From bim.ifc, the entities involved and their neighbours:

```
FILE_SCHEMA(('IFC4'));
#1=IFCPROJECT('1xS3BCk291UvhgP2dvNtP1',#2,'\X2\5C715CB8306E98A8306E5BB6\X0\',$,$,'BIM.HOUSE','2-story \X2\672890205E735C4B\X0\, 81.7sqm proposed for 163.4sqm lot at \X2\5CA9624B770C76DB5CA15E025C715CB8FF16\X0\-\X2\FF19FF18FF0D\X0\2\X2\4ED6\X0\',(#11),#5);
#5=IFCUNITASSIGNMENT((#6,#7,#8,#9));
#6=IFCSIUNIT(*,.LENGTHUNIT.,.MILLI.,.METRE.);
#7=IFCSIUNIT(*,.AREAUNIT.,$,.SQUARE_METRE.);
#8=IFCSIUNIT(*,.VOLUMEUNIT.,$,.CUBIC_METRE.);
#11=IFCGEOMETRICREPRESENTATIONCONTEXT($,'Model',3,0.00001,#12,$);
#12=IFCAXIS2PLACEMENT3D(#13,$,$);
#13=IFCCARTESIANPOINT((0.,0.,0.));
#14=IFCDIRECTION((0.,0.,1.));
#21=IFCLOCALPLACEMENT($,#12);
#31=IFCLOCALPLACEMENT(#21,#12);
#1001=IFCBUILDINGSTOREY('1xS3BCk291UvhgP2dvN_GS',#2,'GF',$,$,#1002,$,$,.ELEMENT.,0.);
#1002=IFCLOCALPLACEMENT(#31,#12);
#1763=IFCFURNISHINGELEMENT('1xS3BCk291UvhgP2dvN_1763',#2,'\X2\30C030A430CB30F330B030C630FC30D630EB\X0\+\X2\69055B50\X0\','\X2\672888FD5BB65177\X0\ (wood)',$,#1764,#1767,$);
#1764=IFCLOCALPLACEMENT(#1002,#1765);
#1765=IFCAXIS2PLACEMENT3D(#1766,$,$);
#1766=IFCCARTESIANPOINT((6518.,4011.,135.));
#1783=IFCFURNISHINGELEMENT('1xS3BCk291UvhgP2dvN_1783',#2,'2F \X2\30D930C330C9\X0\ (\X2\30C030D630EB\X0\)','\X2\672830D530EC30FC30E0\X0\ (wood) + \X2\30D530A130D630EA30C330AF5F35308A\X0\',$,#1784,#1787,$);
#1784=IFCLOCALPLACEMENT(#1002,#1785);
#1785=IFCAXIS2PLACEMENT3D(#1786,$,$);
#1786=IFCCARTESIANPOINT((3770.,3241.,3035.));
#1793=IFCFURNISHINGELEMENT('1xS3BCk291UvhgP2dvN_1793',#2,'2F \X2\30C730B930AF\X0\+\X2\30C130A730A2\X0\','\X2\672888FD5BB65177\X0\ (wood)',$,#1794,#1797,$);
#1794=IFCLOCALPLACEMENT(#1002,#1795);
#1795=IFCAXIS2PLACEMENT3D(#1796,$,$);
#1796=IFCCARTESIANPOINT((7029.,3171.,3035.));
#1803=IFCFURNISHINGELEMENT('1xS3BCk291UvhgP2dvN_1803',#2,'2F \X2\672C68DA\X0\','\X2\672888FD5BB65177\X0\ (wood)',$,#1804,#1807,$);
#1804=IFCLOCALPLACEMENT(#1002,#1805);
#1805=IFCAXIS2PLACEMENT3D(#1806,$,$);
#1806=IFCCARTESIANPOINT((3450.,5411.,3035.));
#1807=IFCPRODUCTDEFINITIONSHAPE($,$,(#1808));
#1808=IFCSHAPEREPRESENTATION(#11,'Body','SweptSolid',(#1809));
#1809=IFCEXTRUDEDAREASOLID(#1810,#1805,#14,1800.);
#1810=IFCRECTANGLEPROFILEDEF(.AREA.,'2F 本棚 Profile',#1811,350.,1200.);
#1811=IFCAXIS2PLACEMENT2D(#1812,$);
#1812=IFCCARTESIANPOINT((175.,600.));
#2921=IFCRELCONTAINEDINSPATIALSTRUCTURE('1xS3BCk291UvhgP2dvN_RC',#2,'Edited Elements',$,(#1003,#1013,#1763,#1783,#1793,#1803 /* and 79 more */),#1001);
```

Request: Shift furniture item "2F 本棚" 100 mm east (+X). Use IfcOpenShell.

```python
import ifcopenshell
import ifcopenshell.api.geometry
import ifcopenshell.util.placement
import ifcopenshell.util.unit

model = ifcopenshell.open("bim.ifc")
unit_scale = ifcopenshell.util.unit.calculate_unit_scale(model)

item = model.by_guid("1xS3BCk291UvhgP2dvN_1803")
matrix = ifcopenshell.util.placement.get_local_placement(item.ObjectPlacement)
matrix[0, 3] += 0.1 / unit_scale
ifcopenshell.api.geometry.edit_object_placement(model, product=item, matrix=matrix, is_si=False)

print(ifcopenshell.util.placement.get_local_placement(item.ObjectPlacement).round(3) + 0.0)

model.write("bim-out.ifc")
```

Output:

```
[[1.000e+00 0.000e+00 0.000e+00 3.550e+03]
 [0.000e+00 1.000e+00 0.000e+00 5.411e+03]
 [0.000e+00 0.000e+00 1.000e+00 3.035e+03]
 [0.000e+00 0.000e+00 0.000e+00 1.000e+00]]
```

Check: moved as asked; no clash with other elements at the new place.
